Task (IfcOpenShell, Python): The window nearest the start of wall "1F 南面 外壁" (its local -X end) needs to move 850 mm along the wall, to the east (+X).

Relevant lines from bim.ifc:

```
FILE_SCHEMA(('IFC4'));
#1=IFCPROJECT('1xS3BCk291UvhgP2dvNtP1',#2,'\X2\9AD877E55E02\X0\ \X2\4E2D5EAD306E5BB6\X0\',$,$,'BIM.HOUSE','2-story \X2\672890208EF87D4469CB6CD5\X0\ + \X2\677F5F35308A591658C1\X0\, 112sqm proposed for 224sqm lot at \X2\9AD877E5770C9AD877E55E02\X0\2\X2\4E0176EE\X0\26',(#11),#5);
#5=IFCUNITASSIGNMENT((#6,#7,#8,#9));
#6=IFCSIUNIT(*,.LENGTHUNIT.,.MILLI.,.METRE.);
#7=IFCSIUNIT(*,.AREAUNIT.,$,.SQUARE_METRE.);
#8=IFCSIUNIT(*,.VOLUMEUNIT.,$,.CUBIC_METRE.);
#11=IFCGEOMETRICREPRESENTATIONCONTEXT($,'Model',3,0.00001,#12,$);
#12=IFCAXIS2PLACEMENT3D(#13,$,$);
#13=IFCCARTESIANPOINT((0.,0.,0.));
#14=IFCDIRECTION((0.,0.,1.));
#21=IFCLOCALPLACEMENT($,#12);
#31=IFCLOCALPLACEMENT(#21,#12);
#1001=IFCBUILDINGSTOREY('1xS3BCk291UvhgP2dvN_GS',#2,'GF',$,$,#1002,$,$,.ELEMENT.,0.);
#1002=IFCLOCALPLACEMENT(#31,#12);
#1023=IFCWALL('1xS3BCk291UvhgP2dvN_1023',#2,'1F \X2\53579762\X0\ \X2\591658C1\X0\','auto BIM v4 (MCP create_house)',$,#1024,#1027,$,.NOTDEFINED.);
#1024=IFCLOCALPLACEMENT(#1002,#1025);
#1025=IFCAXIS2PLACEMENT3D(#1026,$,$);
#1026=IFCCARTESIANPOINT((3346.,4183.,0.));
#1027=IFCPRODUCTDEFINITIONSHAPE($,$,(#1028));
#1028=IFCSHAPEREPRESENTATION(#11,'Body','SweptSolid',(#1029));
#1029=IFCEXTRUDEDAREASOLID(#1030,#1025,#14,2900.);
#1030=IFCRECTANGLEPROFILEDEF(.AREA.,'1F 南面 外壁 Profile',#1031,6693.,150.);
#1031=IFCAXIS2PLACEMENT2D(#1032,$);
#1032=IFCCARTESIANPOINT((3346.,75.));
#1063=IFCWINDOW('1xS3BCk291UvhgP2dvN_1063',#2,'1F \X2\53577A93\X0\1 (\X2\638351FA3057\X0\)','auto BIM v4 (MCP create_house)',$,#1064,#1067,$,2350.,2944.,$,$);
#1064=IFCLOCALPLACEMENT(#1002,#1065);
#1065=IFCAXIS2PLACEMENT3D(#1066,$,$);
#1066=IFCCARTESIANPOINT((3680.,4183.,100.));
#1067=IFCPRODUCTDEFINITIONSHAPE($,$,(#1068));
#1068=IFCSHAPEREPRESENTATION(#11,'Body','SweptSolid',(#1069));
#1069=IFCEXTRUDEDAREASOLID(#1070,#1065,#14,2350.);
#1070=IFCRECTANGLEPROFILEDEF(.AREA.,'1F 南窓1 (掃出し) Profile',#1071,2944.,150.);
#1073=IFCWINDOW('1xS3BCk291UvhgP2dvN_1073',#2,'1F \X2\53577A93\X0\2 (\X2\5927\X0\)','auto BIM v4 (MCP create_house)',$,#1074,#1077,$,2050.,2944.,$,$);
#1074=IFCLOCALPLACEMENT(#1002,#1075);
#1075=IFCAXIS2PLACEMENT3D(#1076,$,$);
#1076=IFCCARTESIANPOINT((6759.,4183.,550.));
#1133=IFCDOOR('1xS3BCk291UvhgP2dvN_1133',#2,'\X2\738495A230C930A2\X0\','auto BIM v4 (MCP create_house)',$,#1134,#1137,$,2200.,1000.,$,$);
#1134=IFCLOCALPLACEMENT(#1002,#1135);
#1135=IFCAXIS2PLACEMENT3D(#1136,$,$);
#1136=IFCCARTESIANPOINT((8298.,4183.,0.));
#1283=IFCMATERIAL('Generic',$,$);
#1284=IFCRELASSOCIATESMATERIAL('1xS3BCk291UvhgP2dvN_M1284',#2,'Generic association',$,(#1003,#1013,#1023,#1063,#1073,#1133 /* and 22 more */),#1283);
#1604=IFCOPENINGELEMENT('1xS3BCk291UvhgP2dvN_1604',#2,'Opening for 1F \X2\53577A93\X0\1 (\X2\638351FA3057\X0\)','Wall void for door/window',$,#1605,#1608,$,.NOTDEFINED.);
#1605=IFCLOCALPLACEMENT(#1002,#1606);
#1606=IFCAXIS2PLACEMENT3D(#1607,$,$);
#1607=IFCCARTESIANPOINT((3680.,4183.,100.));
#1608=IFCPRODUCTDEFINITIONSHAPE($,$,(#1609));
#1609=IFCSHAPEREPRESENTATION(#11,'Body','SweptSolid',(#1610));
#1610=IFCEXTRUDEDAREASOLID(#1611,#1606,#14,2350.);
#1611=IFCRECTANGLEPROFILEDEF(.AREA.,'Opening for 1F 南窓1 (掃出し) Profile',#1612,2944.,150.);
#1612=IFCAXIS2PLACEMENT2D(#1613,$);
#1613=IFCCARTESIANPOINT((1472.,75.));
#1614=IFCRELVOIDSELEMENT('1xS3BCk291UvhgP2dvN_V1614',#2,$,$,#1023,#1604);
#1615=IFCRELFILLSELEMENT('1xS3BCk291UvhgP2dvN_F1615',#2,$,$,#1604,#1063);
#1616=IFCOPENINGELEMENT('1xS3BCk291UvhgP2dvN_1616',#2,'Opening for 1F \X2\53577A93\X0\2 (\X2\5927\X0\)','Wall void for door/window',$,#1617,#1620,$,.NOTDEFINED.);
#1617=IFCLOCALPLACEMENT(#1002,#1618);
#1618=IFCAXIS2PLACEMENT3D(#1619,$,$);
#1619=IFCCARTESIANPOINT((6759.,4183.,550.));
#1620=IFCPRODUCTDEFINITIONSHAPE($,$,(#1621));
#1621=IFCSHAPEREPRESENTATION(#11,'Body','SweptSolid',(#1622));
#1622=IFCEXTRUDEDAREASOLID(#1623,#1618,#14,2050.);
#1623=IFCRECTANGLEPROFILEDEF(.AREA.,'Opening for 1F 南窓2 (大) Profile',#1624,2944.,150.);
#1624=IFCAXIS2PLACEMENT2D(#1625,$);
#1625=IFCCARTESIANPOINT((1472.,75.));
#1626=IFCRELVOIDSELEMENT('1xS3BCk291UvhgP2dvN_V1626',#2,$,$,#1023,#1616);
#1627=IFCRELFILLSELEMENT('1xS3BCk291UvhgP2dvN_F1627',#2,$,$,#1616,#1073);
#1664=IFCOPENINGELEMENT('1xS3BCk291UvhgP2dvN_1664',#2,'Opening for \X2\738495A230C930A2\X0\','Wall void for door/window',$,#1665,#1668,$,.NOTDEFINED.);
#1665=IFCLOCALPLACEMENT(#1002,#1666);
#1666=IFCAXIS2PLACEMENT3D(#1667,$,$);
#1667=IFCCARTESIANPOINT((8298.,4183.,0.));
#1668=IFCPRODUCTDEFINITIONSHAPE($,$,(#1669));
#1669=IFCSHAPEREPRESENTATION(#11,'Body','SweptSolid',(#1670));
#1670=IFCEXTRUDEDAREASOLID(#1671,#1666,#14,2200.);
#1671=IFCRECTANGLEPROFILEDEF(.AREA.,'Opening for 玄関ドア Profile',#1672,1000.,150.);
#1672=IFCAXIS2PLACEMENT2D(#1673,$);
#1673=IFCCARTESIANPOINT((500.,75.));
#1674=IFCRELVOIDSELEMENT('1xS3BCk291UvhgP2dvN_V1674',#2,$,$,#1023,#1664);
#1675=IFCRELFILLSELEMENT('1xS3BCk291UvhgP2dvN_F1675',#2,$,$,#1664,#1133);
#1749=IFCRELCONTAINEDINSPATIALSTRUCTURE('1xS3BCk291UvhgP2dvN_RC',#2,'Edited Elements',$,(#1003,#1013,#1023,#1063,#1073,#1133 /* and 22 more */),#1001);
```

```python
import ifcopenshell
import ifcopenshell.api.geometry
import ifcopenshell.util.placement
import ifcopenshell.util.unit

model = ifcopenshell.open("bim.ifc")
unit_scale = ifcopenshell.util.unit.calculate_unit_scale(model)

window = model.by_guid("1xS3BCk291UvhgP2dvN_1063")
opening = window.FillsVoids[0].RelatingOpeningElement
wall = opening.VoidsElements[0].RelatingBuildingElement

wall_matrix = ifcopenshell.util.placement.get_local_placement(wall.ObjectPlacement)
shift = wall_matrix[:3, 0] * 0.85 / unit_scale
before = ifcopenshell.util.placement.get_local_placement(window.ObjectPlacement)[:3, 3].copy()

# The window is not placed relative to its opening, so move both.
for product in (opening, window):
    matrix = ifcopenshell.util.placement.get_local_placement(product.ObjectPlacement)
    matrix[:3, 3] += shift
    ifcopenshell.api.geometry.edit_object_placement(model, product=product, matrix=matrix, is_si=False)

after = ifcopenshell.util.placement.get_local_placement(window.ObjectPlacement)[:3, 3]
print("window moved by", (after - before).round(3) + 0.0)

model.write("bim_rev.ifc")
```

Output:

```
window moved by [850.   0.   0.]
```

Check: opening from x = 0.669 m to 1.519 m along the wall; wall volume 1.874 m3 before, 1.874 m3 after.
